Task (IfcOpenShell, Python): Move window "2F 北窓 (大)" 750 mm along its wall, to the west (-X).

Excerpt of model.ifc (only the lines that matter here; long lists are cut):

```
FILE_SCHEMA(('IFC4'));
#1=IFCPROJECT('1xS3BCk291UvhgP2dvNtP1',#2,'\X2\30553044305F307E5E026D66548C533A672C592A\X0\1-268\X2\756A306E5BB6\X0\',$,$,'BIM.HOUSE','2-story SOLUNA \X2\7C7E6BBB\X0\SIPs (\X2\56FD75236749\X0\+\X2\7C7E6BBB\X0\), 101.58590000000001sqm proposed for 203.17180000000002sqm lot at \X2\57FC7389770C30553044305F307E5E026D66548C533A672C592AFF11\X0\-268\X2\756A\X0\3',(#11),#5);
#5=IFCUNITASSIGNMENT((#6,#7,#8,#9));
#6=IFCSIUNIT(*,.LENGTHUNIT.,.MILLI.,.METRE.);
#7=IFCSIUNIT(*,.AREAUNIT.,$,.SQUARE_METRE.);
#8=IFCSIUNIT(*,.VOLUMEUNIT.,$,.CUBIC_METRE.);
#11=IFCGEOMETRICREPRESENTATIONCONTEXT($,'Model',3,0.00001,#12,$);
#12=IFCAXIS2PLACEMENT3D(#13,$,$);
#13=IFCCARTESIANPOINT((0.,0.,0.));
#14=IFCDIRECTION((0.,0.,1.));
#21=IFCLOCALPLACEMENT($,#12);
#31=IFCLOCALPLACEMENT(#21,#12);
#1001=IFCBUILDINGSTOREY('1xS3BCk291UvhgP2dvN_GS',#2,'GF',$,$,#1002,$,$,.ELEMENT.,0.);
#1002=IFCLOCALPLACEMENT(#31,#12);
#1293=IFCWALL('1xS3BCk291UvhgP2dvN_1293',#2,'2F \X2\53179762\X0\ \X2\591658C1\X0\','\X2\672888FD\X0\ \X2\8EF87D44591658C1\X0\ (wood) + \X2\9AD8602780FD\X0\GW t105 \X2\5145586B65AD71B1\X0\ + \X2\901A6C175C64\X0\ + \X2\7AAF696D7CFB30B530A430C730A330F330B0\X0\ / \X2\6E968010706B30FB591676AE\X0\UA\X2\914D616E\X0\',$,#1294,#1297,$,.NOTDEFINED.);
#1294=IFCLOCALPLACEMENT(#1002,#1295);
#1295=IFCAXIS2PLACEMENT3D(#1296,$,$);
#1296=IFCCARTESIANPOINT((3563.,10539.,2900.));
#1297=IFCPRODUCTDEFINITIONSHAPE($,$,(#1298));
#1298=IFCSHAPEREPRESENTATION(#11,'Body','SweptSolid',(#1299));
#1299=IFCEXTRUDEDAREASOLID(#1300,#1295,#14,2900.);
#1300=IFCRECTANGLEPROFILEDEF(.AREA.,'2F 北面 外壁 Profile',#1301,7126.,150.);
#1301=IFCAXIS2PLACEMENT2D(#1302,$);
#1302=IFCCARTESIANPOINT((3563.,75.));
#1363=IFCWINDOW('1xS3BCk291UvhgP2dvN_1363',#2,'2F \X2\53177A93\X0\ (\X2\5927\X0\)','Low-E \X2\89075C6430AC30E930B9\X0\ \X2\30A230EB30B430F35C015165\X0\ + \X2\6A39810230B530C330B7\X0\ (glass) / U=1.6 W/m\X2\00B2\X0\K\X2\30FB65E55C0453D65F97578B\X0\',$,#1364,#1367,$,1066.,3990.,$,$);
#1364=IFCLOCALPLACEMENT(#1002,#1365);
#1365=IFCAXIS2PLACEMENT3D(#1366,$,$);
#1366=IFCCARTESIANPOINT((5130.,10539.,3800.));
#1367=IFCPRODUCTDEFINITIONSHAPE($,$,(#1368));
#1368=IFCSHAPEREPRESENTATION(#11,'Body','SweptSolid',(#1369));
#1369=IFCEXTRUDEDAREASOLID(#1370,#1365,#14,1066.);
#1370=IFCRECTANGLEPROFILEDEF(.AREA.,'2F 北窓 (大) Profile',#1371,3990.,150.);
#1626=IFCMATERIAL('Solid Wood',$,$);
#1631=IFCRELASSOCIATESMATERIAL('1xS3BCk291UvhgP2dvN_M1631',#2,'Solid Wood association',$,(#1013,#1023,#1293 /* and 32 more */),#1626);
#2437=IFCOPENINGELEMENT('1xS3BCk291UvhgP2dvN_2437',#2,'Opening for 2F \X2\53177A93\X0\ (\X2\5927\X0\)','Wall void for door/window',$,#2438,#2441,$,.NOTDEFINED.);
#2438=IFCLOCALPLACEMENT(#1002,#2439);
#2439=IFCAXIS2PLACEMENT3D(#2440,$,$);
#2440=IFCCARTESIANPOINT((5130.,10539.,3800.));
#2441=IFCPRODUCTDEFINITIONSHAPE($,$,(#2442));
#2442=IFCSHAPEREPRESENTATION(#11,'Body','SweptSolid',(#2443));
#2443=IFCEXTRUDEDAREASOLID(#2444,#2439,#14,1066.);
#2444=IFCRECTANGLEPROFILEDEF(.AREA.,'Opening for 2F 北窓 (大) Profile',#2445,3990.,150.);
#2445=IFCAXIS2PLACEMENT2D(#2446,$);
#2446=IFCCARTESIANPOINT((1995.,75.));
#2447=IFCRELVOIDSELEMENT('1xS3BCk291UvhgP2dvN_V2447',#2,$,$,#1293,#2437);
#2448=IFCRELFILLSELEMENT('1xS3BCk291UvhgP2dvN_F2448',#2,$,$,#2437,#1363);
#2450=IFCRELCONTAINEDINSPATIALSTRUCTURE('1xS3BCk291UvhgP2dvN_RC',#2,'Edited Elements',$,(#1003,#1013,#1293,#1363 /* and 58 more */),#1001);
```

```python
import ifcopenshell
import ifcopenshell.api.geometry
import ifcopenshell.util.placement
import ifcopenshell.util.unit

model = ifcopenshell.open("model.ifc")
unit_scale = ifcopenshell.util.unit.calculate_unit_scale(model)

window = model.by_id(1363)
opening = window.FillsVoids[0].RelatingOpeningElement
wall = opening.VoidsElements[0].RelatingBuildingElement

wall_matrix = ifcopenshell.util.placement.get_local_placement(wall.ObjectPlacement)
shift = wall_matrix[:3, 0] * -0.75 / unit_scale
before = ifcopenshell.util.placement.get_local_placement(window.ObjectPlacement)[:3, 3].copy()

# The window is not placed relative to its opening, so move both.
for product in (opening, window):
    matrix = ifcopenshell.util.placement.get_local_placement(product.ObjectPlacement)
    matrix[:3, 3] += shift
    ifcopenshell.api.geometry.edit_object_placement(model, product=product, matrix=matrix, is_si=False)

after = ifcopenshell.util.placement.get_local_placement(window.ObjectPlacement)[:3, 3]
print("window moved by", (after - before).round(3) + 0.0)

model.write("model_updated.ifc")
```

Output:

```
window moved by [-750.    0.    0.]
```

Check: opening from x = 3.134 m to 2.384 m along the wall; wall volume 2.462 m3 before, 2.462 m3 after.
